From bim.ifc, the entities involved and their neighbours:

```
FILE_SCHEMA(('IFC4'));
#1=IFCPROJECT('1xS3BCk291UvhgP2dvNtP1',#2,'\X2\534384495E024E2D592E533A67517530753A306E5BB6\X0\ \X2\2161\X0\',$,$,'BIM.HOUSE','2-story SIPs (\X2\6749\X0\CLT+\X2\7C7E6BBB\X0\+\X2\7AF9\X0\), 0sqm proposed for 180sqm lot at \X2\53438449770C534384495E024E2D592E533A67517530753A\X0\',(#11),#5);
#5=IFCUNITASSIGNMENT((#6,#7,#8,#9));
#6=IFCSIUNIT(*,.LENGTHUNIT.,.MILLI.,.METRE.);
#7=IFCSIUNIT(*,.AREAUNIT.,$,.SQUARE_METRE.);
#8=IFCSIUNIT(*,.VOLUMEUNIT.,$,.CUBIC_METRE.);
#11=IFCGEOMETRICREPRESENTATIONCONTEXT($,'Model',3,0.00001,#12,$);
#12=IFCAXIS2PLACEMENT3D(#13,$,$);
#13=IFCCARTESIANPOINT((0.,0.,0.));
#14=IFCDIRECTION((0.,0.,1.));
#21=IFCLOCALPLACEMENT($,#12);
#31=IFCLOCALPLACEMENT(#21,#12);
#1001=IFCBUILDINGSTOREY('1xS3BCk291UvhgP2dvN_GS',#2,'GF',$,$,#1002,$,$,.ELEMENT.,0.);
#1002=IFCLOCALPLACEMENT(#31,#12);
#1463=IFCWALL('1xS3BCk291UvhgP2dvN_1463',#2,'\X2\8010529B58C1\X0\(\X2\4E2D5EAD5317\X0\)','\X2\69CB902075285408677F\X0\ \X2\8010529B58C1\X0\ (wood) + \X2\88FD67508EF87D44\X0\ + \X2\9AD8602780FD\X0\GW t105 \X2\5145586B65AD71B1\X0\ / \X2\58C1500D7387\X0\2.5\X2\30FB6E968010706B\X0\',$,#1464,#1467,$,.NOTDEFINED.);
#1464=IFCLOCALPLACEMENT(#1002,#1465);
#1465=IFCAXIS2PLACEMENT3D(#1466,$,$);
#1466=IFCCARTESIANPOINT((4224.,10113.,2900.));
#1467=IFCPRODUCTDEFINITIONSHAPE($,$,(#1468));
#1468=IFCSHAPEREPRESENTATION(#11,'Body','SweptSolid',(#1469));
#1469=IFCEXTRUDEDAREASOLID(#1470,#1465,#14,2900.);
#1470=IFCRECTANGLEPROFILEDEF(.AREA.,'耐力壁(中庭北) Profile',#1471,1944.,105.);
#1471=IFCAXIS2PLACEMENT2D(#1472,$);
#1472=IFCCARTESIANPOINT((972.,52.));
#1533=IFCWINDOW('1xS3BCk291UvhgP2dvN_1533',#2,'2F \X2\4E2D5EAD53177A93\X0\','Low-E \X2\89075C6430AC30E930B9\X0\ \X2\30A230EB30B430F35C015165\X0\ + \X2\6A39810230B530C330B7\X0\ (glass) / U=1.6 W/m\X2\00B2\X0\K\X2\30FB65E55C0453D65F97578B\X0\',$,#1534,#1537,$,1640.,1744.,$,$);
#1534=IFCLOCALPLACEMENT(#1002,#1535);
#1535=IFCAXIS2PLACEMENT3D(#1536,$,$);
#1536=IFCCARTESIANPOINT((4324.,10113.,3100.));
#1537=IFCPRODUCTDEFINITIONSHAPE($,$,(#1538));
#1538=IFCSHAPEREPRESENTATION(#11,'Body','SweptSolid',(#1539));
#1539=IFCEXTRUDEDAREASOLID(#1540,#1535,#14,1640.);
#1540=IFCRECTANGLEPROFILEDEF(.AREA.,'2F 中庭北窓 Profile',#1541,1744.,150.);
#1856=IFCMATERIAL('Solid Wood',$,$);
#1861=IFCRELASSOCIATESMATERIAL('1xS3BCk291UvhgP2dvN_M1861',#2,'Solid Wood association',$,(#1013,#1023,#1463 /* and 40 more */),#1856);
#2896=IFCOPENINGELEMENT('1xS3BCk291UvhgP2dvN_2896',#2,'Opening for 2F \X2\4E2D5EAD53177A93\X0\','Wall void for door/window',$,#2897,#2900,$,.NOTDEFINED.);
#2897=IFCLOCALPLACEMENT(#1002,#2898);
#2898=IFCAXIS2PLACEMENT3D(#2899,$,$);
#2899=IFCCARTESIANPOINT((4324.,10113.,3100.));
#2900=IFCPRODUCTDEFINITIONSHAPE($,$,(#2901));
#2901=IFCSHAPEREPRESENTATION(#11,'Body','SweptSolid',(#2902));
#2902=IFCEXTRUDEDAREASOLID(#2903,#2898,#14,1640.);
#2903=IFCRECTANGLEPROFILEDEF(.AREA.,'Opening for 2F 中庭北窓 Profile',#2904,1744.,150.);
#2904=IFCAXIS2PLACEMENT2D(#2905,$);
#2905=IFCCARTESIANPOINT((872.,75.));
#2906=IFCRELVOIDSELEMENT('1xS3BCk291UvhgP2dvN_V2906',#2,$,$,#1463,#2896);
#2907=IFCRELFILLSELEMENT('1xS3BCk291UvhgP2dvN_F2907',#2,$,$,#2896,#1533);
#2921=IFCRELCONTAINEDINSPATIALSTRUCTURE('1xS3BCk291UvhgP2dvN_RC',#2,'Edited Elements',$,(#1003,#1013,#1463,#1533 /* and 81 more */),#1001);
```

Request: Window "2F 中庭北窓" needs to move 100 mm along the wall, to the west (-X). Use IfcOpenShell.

```python
import ifcopenshell
import ifcopenshell.api.geometry
import ifcopenshell.util.placement
import ifcopenshell.util.unit

model = ifcopenshell.open("bim.ifc")
unit_scale = ifcopenshell.util.unit.calculate_unit_scale(model)

window = model.by_guid("1xS3BCk291UvhgP2dvN_1533")
opening = window.FillsVoids[0].RelatingOpeningElement
wall = opening.VoidsElements[0].RelatingBuildingElement

wall_matrix = ifcopenshell.util.placement.get_local_placement(wall.ObjectPlacement)
shift = wall_matrix[:3, 0] * -0.1 / unit_scale
before = ifcopenshell.util.placement.get_local_placement(window.ObjectPlacement)[:3, 3].copy()

# The window is not placed relative to its opening, so move both.
for product in (opening, window):
    matrix = ifcopenshell.util.placement.get_local_placement(product.ObjectPlacement)
    matrix[:3, 3] += shift
    ifcopenshell.api.geometry.edit_object_placement(model, product=product, matrix=matrix, is_si=False)

after = ifcopenshell.util.placement.get_local_placement(window.ObjectPlacement)[:3, 3]
print("window moved by", (after - before).round(3) + 0.0)

model.write("bim_updated.ifc")
```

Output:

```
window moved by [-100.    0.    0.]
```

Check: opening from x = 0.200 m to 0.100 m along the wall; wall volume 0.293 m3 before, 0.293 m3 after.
